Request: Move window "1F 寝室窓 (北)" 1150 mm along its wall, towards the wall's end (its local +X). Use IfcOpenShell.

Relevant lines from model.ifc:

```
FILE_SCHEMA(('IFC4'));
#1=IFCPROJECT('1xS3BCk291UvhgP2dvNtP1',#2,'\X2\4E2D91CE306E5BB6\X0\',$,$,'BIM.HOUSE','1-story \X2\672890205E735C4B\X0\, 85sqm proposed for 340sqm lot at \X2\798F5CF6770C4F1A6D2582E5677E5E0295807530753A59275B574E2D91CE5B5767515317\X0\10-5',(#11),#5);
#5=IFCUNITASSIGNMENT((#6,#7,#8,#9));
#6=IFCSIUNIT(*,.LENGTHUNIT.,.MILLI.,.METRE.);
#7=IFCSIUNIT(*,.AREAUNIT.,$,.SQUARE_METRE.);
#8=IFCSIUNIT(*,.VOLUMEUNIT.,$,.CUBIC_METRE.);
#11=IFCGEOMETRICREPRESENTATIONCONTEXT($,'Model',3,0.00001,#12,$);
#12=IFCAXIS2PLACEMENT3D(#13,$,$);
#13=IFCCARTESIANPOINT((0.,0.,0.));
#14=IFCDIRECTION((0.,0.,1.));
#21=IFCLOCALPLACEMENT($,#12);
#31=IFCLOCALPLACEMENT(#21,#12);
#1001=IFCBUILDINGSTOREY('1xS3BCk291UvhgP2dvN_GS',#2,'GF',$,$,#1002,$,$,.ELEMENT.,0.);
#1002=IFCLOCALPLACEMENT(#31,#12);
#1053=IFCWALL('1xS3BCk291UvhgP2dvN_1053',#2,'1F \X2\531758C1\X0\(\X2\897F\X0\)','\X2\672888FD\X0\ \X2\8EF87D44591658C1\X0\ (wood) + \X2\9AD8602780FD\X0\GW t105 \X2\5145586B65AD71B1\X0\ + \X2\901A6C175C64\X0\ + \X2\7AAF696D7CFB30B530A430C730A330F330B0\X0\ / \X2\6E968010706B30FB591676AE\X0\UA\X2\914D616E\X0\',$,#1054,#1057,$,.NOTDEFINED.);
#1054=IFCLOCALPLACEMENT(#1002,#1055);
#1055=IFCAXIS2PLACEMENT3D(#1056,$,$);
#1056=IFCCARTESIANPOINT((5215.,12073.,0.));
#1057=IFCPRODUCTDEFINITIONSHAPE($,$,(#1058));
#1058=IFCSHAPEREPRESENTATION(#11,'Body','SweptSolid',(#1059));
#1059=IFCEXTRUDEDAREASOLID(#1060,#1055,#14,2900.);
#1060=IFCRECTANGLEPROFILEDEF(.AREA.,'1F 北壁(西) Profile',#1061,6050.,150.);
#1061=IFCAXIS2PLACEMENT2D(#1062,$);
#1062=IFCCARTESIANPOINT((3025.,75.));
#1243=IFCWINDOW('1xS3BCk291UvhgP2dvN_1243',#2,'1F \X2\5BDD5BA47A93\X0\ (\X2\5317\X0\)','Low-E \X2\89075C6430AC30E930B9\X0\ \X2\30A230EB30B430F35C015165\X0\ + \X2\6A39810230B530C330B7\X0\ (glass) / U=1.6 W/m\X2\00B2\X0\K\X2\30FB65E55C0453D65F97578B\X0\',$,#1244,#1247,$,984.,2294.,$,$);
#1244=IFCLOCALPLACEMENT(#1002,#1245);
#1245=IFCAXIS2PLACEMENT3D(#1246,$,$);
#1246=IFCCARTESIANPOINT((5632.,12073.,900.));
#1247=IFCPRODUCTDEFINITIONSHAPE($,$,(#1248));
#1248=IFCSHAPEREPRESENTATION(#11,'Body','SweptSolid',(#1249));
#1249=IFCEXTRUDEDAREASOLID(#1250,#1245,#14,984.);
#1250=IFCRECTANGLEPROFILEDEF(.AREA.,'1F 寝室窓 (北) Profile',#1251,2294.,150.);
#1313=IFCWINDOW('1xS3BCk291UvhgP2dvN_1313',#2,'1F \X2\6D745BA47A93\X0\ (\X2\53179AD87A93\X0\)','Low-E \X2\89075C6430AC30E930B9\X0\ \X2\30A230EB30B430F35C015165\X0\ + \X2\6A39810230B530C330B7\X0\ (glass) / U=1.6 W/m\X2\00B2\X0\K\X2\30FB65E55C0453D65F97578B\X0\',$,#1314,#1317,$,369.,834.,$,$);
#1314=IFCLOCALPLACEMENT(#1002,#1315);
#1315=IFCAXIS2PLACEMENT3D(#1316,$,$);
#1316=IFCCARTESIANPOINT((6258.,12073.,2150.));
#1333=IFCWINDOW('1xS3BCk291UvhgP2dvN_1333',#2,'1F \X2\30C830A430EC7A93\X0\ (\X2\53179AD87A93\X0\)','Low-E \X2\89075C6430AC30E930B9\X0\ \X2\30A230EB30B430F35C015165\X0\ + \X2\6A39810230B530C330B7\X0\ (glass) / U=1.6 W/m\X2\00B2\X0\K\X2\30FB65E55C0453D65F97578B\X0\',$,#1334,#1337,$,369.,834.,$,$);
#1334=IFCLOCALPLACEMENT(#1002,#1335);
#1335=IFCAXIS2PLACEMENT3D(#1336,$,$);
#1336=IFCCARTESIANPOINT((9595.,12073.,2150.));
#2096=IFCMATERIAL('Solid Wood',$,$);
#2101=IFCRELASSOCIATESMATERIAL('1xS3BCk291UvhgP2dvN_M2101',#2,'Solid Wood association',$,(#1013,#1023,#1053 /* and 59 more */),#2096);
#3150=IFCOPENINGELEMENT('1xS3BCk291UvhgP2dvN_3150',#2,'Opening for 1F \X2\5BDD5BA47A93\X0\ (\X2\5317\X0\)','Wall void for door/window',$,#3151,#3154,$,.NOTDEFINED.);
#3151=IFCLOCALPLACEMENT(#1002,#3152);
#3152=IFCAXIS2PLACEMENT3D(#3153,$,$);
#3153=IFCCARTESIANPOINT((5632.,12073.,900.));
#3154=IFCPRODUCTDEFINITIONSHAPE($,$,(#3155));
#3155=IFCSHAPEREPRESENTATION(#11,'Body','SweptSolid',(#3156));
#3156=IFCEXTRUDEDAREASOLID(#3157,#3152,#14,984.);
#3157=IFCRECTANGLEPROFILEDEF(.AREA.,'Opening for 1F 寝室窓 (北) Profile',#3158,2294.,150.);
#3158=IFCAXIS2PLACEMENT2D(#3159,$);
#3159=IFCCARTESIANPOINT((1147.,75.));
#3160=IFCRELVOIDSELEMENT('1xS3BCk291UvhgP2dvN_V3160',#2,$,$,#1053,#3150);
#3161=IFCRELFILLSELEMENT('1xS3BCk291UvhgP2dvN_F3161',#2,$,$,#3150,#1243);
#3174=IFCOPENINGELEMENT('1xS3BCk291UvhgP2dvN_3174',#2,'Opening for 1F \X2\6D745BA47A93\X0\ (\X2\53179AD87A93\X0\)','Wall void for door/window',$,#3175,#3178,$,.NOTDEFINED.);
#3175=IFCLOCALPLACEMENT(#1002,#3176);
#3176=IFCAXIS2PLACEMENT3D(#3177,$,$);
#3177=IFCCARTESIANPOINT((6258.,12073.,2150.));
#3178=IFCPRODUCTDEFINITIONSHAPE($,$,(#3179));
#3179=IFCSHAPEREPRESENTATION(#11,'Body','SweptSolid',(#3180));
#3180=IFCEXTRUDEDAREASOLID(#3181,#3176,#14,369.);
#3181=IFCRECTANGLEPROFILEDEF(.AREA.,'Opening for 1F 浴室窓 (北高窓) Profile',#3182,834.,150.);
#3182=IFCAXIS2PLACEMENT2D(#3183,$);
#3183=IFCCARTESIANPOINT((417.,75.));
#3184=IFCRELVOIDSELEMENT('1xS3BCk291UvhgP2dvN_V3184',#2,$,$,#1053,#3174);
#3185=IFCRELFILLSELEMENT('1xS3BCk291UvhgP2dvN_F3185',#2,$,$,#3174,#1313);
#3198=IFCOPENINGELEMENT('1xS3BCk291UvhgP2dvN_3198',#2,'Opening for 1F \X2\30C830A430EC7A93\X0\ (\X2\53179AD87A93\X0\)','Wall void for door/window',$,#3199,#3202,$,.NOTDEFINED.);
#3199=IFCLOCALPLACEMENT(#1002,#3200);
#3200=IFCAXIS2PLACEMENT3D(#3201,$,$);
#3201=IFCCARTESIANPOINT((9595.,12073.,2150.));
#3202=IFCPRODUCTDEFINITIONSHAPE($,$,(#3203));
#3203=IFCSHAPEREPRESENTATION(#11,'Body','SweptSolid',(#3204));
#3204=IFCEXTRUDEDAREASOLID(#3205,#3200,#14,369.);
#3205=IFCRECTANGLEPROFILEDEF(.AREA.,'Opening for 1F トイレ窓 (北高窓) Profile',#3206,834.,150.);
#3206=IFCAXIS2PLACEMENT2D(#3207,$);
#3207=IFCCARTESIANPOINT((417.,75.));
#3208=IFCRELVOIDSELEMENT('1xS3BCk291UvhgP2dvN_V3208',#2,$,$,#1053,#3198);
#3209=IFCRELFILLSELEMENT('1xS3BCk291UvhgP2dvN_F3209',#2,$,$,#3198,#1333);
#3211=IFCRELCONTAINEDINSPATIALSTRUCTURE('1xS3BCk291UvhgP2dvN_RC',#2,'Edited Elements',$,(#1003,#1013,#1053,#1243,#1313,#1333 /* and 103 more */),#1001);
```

```python
import ifcopenshell
import ifcopenshell.api.geometry
import ifcopenshell.util.placement

model = ifcopenshell.open("model.ifc")

window = model.by_guid("1xS3BCk291UvhgP2dvN_1243")
opening = window.FillsVoids[0].RelatingOpeningElement
wall = opening.VoidsElements[0].RelatingBuildingElement

wall_matrix = ifcopenshell.util.placement.get_local_placement(wall.ObjectPlacement)
shift = wall_matrix[:3, 0] * 1150.0
before = ifcopenshell.util.placement.get_local_placement(window.ObjectPlacement)[:3, 3].copy()

# The window is not placed relative to its opening, so move both.
for product in (opening, window):
    matrix = ifcopenshell.util.placement.get_local_placement(product.ObjectPlacement)
    matrix[:3, 3] += shift
    ifcopenshell.api.geometry.edit_object_placement(model, product=product, matrix=matrix, is_si=False)

after = ifcopenshell.util.placement.get_local_placement(window.ObjectPlacement)[:3, 3]
print("window moved by", (after - before).round(3) + 0.0)

model.write("model-out.ifc")
```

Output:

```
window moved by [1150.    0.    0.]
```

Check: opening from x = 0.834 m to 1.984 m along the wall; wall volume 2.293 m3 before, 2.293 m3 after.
